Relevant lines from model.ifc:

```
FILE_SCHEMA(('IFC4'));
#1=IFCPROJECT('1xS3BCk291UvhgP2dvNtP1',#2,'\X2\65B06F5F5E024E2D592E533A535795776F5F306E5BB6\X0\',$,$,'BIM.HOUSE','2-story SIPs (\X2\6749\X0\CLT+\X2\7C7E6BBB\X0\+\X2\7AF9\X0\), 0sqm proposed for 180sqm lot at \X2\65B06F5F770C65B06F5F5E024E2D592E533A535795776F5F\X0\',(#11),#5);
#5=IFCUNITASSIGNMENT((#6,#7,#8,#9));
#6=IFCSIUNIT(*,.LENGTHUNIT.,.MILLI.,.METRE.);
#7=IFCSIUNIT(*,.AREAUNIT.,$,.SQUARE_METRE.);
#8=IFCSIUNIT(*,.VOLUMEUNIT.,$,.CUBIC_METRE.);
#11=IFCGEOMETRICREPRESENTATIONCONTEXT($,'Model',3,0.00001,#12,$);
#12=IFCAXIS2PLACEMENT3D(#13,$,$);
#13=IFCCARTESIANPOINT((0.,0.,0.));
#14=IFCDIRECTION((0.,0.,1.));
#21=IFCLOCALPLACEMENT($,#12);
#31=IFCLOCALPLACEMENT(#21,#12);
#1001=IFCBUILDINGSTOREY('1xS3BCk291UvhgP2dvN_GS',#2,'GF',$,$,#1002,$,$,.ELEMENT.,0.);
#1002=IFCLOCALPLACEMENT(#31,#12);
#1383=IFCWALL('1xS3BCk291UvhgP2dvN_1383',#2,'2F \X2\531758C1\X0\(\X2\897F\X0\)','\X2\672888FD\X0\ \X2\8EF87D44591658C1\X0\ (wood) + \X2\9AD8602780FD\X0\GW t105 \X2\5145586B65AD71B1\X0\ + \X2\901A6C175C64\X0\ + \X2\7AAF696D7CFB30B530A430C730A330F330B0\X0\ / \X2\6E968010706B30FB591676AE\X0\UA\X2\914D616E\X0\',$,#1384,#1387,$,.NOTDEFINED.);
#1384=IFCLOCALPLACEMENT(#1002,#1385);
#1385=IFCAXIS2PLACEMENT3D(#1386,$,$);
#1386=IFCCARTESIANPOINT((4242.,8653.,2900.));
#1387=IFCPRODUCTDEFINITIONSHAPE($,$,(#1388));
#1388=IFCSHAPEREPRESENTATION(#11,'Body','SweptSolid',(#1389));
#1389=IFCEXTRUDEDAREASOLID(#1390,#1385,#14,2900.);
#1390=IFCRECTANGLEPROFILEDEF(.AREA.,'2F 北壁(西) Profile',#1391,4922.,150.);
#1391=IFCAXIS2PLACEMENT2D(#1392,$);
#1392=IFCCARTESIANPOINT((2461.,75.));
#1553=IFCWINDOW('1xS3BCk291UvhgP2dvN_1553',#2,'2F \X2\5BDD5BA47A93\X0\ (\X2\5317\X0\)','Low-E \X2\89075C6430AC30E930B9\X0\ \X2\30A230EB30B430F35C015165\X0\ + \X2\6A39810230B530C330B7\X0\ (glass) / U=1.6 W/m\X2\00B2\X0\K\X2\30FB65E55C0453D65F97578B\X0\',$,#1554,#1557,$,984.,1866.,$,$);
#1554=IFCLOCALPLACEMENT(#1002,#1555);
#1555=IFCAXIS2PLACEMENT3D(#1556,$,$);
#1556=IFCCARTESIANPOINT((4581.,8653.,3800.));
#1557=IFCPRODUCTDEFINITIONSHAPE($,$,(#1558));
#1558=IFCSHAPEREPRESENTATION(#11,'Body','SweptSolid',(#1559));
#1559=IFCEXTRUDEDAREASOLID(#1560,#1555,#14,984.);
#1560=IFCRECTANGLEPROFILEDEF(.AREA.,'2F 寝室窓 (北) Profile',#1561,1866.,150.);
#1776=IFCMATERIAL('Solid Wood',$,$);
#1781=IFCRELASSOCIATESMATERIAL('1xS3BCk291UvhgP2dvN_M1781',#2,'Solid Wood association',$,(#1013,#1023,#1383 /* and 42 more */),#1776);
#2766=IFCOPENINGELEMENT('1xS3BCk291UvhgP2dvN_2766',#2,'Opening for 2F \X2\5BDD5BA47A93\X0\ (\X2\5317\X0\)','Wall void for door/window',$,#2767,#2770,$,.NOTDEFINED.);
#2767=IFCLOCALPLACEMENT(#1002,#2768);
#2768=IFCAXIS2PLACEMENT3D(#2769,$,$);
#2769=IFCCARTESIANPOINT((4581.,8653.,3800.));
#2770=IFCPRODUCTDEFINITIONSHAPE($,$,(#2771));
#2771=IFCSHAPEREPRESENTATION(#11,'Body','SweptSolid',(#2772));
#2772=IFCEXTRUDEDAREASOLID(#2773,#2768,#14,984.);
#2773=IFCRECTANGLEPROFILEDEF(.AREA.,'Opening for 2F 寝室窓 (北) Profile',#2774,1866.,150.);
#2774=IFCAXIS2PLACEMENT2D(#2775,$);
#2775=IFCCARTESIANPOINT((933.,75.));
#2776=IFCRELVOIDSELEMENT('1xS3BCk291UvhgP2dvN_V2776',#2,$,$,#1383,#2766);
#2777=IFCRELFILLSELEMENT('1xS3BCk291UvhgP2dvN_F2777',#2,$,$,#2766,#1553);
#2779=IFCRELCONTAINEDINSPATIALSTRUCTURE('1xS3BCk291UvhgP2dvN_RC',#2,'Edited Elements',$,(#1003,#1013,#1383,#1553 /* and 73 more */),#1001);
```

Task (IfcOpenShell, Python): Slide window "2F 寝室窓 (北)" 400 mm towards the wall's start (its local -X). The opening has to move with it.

```python
import ifcopenshell
import ifcopenshell.api.geometry
import ifcopenshell.util.placement

model = ifcopenshell.open("model.ifc")

window = model.by_guid("1xS3BCk291UvhgP2dvN_1553")
opening = window.FillsVoids[0].RelatingOpeningElement
wall = opening.VoidsElements[0].RelatingBuildingElement

wall_matrix = ifcopenshell.util.placement.get_local_placement(wall.ObjectPlacement)
shift = wall_matrix[:3, 0] * -400.0
before = ifcopenshell.util.placement.get_local_placement(window.ObjectPlacement)[:3, 3].copy()

# The window is not placed relative to its opening, so move both.
for product in (opening, window):
    matrix = ifcopenshell.util.placement.get_local_placement(product.ObjectPlacement)
    matrix[:3, 3] += shift
    ifcopenshell.api.geometry.edit_object_placement(model, product=product, matrix=matrix, is_si=False)

after = ifcopenshell.util.placement.get_local_placement(window.ObjectPlacement)[:3, 3]
print("window moved by", (after - before).round(3) + 0.0)

model.write("model_edited.ifc")
```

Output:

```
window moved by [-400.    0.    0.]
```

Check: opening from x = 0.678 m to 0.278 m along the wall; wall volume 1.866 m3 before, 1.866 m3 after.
